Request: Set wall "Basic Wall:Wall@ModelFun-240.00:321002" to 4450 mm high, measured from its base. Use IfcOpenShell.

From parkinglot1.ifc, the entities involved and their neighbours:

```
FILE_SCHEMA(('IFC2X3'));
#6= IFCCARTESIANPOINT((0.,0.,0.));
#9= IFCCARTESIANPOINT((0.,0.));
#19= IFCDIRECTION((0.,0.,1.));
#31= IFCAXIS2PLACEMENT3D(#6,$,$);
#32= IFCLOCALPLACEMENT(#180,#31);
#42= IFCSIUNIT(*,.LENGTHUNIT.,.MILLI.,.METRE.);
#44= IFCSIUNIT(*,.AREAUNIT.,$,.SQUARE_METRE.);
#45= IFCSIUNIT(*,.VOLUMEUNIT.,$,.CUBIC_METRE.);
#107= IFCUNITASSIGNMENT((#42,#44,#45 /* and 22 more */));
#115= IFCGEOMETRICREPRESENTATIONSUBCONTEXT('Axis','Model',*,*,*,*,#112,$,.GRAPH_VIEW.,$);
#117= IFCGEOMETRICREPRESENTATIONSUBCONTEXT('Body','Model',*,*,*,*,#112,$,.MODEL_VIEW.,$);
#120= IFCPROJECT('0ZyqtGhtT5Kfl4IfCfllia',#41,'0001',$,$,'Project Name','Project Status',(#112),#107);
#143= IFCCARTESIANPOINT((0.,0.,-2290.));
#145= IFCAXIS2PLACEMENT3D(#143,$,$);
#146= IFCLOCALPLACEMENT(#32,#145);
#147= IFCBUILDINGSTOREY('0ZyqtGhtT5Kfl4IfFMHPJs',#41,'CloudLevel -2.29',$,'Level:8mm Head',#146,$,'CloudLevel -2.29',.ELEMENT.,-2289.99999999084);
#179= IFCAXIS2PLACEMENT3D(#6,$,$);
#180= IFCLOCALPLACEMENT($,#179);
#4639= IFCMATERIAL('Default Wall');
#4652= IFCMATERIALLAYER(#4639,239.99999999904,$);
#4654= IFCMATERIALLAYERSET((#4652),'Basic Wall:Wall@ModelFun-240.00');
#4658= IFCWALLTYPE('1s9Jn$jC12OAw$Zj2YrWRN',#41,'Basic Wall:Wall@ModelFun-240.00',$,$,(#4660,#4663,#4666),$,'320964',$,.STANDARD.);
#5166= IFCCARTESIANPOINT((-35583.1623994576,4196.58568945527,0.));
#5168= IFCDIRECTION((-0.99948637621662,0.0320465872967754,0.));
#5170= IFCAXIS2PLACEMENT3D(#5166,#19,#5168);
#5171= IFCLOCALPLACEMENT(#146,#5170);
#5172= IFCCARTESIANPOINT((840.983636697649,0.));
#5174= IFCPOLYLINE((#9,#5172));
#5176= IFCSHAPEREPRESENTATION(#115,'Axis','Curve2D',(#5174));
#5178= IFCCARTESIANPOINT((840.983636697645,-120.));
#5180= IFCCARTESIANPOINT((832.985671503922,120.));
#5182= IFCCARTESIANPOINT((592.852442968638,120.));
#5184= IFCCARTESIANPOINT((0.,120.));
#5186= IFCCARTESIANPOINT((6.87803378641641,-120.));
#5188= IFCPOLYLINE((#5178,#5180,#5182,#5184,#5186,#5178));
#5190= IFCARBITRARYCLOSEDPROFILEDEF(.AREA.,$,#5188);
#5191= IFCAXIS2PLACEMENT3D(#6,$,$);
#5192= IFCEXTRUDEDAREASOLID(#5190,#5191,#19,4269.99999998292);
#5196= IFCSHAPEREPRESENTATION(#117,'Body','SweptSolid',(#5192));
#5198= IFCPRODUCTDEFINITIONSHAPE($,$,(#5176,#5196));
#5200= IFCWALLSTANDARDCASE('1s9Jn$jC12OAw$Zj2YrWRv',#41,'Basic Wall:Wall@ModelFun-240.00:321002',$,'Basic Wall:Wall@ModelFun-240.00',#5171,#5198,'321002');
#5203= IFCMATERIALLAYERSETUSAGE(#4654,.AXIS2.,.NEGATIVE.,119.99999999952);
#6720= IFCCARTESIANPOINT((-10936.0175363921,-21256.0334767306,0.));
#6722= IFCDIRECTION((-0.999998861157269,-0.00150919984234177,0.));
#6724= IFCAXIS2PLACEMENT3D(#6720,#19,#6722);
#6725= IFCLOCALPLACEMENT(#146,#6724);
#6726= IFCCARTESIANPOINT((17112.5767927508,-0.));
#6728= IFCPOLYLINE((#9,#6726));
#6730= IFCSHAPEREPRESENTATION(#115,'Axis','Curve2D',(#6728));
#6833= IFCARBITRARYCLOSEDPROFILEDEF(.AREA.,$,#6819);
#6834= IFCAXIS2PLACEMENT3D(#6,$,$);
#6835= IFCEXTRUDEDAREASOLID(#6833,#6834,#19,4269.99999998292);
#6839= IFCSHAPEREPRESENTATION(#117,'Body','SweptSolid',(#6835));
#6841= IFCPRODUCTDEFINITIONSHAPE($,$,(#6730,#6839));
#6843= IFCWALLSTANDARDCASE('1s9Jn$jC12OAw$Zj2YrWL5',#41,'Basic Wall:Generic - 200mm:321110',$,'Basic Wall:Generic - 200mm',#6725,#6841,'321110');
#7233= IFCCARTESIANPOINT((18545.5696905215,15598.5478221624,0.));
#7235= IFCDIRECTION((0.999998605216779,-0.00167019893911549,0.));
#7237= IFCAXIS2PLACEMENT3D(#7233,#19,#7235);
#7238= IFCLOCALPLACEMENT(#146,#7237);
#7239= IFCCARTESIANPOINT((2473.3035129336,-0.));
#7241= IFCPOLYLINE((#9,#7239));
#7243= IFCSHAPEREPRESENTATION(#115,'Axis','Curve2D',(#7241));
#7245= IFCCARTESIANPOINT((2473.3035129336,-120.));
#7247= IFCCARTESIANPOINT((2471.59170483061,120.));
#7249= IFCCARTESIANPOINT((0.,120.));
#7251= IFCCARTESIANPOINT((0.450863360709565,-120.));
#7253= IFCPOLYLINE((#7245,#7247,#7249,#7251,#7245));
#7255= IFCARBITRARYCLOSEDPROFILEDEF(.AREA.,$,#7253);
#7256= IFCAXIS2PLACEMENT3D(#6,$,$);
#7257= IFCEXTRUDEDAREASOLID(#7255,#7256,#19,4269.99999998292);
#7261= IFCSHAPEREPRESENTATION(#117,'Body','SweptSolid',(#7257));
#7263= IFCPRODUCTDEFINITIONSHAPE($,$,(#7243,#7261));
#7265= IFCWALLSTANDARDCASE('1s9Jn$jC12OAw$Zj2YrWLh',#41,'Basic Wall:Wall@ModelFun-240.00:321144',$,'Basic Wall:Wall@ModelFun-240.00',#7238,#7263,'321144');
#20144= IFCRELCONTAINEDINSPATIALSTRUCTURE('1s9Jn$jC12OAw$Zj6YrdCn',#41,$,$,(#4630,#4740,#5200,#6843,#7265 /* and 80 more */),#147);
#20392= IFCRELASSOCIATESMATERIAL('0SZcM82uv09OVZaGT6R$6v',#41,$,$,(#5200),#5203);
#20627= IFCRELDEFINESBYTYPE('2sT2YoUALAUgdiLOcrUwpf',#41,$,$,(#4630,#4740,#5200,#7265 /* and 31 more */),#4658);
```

```python
import ifcopenshell
import ifcopenshell.geom
import ifcopenshell.util.representation
import ifcopenshell.util.shape
import ifcopenshell.util.unit

model = ifcopenshell.open("parkinglot1.ifc")
unit_scale = ifcopenshell.util.unit.calculate_unit_scale(model)
settings = ifcopenshell.geom.settings()


def volume(element):
    """Net volume in cubic metres, openings subtracted."""
    shape = ifcopenshell.geom.create_shape(settings, element)
    return ifcopenshell.util.shape.get_volume(shape.geometry)


wall = model.by_id(5200)
before = volume(wall)

body = ifcopenshell.util.representation.get_representation(wall, "Model", "Body")
solid = body.Items[0]
old_height = solid.Depth
solid.Depth = 4.45 / unit_scale
after = volume(wall)

print(f"height {old_height:g} -> {solid.Depth:g}, volume {before:.3f} -> {after:.3f} m3")

model.write("parkinglot1_rev.ifc")
```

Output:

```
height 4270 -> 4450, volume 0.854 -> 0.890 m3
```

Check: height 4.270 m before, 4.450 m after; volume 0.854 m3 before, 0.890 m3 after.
